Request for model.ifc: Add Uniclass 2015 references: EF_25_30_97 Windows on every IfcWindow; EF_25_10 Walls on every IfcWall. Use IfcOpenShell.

First a look at what the model holds.

```python
import ifcopenshell

model = ifcopenshell.open("model.ifc")
print(model.schema)
print("classifications:", [c.Name for c in model.by_type("IfcClassification")])
for ifc_class in ("IfcDoor", "IfcRoof", "IfcStair", "IfcWall", "IfcWindow"):
    print(ifc_class, len(model.by_type(ifc_class)))
```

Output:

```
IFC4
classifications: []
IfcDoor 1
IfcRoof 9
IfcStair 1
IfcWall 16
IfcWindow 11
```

```python
import ifcopenshell
import ifcopenshell.api.classification

model = ifcopenshell.open("model.ifc")

system = ifcopenshell.api.classification.add_classification(model, classification="Uniclass 2015")

codes = {
    "IfcWindow": ("EF_25_30_97", "Windows"),
    "IfcWall": ("EF_25_10", "Walls"),
}
for ifc_class, (code, name) in codes.items():
    products = model.by_type(ifc_class)
    ifcopenshell.api.classification.add_reference(
        model, products=products, classification=system, identification=code, name=name
    )
    print(code, len(products))

model.write("model-out.ifc")
```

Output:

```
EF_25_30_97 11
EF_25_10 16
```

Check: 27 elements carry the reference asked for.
